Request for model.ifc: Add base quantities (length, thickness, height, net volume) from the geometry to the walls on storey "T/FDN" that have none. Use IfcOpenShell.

First a look at what the model holds.

```python
import ifcopenshell
import ifcopenshell.util.element
import ifcopenshell.util.unit

model = ifcopenshell.open("model.ifc")
print(model.schema)
for unit_type in ("LENGTHUNIT", "AREAUNIT", "VOLUMEUNIT"):
    print(unit_type, ifcopenshell.util.unit.calculate_unit_scale(model, unit_type))
storey = next(s for s in model.by_type("IfcBuildingStorey") if s.Name == "T/FDN")
walls = [e for e in ifcopenshell.util.element.get_decomposition(storey) if e.is_a("IfcWall")]
for e in sorted(walls, key=lambda e: e.id()):
    print(e.id(), e.is_a(), e.Name, list(ifcopenshell.util.element.get_psets(e, qtos_only=True)), sep=" | ")
```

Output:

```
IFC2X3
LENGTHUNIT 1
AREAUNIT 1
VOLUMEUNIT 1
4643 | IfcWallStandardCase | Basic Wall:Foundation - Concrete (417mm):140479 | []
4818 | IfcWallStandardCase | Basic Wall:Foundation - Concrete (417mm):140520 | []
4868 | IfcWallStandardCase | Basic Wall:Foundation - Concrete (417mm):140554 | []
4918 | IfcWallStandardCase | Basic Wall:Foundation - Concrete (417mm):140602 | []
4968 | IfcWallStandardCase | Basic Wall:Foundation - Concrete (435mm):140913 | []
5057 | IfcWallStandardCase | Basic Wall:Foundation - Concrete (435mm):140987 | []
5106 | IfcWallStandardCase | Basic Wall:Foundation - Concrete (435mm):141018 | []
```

```python
import ifcopenshell
import ifcopenshell.api.pset
import ifcopenshell.geom
import ifcopenshell.util.element
import ifcopenshell.util.shape
import ifcopenshell.util.unit

model = ifcopenshell.open("model.ifc")
unit_scale = ifcopenshell.util.unit.calculate_unit_scale(model)
volume_scale = ifcopenshell.util.unit.calculate_unit_scale(model, "VOLUMEUNIT")
settings = ifcopenshell.geom.settings()

storey = next(s for s in model.by_type("IfcBuildingStorey") if s.Name == "T/FDN")
walls = [e for e in ifcopenshell.util.element.get_decomposition(storey) if e.is_a("IfcWall")]

for e in sorted(walls, key=lambda e: e.id()):
    if ifcopenshell.util.element.get_psets(e, qtos_only=True, should_inherit=False):
        continue
    # Geometry comes back in metres, in the element's own axes.
    shape = ifcopenshell.geom.create_shape(settings, e)
    values = {
        "Length": ifcopenshell.util.shape.get_x(shape.geometry) / unit_scale,
        "Width": ifcopenshell.util.shape.get_y(shape.geometry) / unit_scale,
        "Height": ifcopenshell.util.shape.get_z(shape.geometry) / unit_scale,
        "NetVolume": ifcopenshell.util.shape.get_volume(shape.geometry) / volume_scale,
    }
    qto = ifcopenshell.api.pset.add_qto(model, product=e, name="BaseQuantities")
    ifcopenshell.api.pset.edit_qto(model, qto=qto, properties=values)
    print(e.id(), {k: round(v, 3) for k, v in values.items()})

model.write("model-out.ifc")
```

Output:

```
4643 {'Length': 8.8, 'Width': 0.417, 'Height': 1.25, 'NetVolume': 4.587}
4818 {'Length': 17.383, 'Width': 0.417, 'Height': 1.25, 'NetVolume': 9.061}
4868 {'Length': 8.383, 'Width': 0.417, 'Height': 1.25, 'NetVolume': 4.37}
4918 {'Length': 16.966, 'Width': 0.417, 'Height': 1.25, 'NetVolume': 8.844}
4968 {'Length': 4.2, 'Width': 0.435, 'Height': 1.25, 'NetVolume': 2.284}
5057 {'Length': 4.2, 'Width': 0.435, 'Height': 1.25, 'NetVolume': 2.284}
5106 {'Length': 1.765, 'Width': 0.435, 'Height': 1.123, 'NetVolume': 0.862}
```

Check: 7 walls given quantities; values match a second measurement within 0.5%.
